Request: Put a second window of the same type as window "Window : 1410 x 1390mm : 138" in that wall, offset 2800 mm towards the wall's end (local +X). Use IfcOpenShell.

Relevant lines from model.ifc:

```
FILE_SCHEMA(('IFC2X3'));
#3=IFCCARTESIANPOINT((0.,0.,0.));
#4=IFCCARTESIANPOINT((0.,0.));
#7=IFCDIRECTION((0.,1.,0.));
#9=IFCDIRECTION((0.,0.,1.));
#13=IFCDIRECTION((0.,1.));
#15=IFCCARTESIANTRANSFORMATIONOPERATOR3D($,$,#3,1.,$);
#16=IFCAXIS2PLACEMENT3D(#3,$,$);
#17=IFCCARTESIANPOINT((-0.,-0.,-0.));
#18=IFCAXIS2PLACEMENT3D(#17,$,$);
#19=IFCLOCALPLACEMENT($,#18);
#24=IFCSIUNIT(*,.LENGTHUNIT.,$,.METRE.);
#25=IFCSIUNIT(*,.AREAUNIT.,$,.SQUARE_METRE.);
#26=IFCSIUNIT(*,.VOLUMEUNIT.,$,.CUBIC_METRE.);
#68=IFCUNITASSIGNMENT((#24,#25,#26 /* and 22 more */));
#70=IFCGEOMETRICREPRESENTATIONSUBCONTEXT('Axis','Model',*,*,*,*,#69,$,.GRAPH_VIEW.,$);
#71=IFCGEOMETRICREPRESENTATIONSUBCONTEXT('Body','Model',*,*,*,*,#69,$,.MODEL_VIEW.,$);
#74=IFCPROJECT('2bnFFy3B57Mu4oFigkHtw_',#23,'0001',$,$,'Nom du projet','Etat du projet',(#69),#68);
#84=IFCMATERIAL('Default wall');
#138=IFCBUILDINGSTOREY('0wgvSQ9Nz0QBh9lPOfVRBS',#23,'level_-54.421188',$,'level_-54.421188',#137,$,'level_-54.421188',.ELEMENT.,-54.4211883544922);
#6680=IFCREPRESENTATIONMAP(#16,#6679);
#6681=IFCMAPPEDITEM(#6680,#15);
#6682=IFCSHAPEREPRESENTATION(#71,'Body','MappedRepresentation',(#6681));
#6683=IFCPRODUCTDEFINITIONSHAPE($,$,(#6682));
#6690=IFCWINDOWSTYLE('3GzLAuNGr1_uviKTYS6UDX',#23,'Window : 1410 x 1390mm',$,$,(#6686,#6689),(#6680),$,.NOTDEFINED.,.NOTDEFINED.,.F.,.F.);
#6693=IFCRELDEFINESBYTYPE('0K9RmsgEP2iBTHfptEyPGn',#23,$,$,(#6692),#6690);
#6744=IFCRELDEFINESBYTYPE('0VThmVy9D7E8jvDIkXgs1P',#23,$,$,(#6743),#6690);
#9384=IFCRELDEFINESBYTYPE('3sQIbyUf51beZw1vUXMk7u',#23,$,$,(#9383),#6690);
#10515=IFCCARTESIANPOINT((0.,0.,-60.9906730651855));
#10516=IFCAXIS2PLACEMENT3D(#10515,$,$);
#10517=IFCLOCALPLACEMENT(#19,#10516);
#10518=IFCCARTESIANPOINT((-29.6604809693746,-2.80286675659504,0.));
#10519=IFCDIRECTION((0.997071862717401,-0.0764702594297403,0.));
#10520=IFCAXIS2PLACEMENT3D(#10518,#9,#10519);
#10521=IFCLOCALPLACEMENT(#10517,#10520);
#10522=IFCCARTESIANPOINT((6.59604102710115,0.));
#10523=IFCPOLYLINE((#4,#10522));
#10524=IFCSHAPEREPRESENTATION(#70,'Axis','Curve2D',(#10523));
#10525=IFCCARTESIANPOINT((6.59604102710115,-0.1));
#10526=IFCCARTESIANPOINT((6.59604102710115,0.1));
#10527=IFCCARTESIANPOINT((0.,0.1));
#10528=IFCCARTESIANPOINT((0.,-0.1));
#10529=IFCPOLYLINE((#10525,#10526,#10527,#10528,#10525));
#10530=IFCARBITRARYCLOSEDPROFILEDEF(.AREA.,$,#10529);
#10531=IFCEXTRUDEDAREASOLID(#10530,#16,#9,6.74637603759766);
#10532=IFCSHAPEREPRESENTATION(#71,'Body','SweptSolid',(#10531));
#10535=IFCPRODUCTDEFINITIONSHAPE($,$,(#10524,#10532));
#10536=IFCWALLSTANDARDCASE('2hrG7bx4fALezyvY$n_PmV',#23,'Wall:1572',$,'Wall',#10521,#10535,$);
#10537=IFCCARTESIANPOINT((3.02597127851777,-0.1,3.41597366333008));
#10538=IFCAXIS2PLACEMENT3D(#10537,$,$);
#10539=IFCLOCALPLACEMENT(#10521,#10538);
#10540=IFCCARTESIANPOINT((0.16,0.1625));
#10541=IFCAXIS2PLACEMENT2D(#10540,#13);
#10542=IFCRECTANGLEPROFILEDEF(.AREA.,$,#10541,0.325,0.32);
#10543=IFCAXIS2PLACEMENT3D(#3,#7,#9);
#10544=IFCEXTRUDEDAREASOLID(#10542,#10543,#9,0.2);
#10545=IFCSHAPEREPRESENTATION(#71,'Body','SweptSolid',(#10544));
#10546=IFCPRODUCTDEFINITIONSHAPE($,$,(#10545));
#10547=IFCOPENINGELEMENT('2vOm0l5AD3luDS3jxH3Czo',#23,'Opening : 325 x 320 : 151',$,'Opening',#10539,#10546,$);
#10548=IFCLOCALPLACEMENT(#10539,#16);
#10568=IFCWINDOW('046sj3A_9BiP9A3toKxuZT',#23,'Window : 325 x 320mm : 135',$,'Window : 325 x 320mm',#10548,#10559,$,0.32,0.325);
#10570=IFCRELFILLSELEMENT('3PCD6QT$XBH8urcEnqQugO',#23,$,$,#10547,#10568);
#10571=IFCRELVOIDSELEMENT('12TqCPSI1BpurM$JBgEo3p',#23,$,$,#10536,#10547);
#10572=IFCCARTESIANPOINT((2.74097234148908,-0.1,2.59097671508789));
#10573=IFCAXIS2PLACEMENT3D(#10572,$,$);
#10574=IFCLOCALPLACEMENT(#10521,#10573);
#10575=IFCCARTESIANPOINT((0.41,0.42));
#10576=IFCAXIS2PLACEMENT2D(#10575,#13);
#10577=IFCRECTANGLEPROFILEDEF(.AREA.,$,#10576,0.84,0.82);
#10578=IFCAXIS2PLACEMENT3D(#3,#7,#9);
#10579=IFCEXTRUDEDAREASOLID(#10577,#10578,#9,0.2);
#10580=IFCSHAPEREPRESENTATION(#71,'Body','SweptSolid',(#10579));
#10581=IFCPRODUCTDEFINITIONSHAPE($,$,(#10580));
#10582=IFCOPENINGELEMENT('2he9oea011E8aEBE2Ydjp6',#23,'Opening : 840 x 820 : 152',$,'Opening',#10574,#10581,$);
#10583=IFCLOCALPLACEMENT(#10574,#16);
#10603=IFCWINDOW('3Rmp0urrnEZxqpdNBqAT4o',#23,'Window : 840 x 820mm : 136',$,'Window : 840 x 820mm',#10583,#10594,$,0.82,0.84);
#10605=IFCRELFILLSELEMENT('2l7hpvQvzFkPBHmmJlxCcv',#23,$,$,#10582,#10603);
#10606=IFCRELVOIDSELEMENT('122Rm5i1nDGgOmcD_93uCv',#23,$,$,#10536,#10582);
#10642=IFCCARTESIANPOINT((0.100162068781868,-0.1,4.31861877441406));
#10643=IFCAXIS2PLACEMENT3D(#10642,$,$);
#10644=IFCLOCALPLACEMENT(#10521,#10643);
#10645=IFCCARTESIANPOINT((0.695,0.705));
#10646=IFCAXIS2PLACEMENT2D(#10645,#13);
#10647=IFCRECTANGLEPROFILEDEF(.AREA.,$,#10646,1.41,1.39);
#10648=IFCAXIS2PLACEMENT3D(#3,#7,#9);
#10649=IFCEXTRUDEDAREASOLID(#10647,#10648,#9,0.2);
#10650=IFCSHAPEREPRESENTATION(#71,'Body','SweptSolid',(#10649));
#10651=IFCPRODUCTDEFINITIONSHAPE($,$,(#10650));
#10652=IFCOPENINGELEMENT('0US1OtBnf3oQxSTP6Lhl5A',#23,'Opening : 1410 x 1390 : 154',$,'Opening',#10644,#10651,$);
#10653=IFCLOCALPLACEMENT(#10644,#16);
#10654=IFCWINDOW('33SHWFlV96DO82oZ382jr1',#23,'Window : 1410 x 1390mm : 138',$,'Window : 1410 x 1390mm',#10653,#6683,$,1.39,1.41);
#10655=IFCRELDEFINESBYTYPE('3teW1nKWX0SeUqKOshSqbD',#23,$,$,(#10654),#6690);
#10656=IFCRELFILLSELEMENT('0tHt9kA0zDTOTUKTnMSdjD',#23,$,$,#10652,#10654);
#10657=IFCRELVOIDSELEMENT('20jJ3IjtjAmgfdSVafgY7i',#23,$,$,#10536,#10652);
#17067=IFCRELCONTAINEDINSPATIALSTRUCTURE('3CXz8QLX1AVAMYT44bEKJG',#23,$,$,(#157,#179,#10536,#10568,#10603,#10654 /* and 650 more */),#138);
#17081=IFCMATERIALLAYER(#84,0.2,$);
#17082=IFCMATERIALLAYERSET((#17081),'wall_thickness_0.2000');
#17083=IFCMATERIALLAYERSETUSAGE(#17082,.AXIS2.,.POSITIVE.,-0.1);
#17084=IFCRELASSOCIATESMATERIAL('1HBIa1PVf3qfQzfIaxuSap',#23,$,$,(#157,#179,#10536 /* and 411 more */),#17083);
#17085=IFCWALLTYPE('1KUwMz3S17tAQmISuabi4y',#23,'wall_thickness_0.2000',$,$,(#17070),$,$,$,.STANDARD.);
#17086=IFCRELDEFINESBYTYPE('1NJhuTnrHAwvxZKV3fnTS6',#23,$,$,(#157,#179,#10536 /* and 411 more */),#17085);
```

```python
import ifcopenshell
import ifcopenshell.api.feature
import ifcopenshell.api.geometry
import ifcopenshell.api.root
import ifcopenshell.geom
import ifcopenshell.util.element
import ifcopenshell.util.placement
import ifcopenshell.util.shape
import ifcopenshell.util.unit

model = ifcopenshell.open("model.ifc")
unit_scale = ifcopenshell.util.unit.calculate_unit_scale(model)
settings = ifcopenshell.geom.settings()


def volume(element):
    """Net volume in cubic metres, openings subtracted."""
    shape = ifcopenshell.geom.create_shape(settings, element)
    return ifcopenshell.util.shape.get_volume(shape.geometry)


window = model.by_guid("33SHWFlV96DO82oZ382jr1")
opening = window.FillsVoids[0].RelatingOpeningElement
wall = opening.VoidsElements[0].RelatingBuildingElement
before = volume(wall)
shift = ifcopenshell.util.placement.get_local_placement(wall.ObjectPlacement)[:3, 0] * 2.8 / unit_scale

# copy_class copies the void relationship, type, container and properties, but no geometry.
new_opening = ifcopenshell.api.root.copy_class(model, product=opening)
new_opening.Representation = ifcopenshell.util.element.copy_deep(
    model, opening.Representation, exclude=["IfcGeometricRepresentationContext", "IfcRepresentationMap"]
)
new_opening.Name = "Opening : 1410 x 1390"
new_window = ifcopenshell.api.root.copy_class(model, product=window)
new_window.Representation = ifcopenshell.util.element.copy_deep(
    model, window.Representation, exclude=["IfcGeometricRepresentationContext", "IfcRepresentationMap"]
)
new_window.Name = "Window : 1410 x 1390mm"
fills = ifcopenshell.api.feature.add_filling(model, opening=new_opening, element=new_window)
fills.OwnerHistory = new_window.OwnerHistory  # required in IFC2X3

for old, new in ((opening, new_opening), (window, new_window)):
    matrix = ifcopenshell.util.placement.get_local_placement(old.ObjectPlacement)
    matrix[:3, 3] += shift
    ifcopenshell.api.geometry.edit_object_placement(model, product=new, matrix=matrix, is_si=False)

after = volume(wall)

print(f"wall volume {before:.3f} -> {after:.3f} m3")

model.write("model_updated.ifc")
```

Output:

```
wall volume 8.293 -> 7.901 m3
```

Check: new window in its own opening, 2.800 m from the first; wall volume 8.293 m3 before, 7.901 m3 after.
